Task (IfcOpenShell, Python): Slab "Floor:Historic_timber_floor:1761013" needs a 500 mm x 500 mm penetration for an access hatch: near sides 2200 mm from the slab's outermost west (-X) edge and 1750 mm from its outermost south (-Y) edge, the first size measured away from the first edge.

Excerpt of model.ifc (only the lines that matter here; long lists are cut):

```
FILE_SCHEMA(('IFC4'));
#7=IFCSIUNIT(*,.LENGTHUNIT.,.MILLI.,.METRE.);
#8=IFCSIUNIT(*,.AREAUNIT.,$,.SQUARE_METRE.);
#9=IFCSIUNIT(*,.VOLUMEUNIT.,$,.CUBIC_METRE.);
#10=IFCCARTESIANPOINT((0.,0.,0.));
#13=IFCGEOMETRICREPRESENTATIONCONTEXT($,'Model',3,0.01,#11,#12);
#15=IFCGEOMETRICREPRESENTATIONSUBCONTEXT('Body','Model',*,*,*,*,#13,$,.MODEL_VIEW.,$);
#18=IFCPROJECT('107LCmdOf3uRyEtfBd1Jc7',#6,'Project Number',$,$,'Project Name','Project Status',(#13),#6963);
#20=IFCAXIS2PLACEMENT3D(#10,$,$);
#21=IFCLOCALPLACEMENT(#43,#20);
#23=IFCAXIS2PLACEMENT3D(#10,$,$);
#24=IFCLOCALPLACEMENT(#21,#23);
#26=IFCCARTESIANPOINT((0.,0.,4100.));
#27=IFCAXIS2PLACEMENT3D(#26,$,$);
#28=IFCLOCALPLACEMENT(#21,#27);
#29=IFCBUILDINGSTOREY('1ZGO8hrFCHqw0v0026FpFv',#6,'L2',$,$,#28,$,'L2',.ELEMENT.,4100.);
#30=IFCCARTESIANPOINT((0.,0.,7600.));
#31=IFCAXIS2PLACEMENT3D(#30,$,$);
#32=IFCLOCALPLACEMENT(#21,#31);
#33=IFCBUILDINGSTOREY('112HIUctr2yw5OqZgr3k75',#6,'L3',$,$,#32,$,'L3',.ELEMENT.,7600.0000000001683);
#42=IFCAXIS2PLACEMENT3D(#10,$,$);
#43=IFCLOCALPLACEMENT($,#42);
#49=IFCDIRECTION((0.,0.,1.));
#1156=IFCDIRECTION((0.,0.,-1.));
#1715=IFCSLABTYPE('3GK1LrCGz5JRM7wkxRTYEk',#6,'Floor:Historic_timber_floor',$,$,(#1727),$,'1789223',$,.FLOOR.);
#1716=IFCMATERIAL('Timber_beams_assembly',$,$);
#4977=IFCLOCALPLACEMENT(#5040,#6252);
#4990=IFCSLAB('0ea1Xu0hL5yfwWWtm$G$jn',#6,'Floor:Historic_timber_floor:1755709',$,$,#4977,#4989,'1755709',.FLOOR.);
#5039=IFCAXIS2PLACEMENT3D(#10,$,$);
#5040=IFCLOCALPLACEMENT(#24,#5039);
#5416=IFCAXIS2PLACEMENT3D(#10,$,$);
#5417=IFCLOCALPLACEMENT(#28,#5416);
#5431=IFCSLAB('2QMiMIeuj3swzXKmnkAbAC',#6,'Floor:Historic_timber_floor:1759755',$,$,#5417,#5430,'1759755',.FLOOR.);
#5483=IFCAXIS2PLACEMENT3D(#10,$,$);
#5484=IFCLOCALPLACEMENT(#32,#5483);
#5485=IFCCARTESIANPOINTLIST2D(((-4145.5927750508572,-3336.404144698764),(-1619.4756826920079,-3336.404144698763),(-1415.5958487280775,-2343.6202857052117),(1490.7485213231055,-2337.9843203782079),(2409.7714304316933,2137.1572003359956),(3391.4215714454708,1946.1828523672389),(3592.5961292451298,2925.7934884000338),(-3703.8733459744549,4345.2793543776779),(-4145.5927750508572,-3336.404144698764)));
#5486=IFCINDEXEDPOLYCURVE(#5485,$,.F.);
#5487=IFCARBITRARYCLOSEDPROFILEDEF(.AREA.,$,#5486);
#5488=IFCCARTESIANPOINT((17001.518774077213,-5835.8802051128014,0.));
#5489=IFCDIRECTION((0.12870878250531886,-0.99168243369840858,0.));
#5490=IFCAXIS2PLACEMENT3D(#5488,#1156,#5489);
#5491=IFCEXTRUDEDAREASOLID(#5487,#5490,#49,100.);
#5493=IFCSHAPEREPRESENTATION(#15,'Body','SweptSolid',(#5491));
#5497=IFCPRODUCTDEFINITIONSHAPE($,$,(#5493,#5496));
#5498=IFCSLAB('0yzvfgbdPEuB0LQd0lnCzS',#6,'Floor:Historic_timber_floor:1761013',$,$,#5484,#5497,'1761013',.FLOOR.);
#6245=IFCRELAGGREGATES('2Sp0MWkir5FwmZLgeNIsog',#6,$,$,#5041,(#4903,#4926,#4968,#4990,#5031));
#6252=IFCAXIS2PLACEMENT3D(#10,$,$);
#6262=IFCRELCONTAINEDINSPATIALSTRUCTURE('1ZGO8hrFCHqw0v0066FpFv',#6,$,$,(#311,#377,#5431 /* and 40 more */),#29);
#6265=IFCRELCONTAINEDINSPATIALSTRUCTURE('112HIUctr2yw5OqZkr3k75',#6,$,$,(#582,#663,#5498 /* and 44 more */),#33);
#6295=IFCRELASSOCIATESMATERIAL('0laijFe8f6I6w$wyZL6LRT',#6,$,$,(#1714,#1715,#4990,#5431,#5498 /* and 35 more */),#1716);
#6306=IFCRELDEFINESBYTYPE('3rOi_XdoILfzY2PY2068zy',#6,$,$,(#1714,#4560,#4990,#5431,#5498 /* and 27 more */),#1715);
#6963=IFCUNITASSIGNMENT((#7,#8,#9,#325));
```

```python
import numpy as np
import ifcopenshell
import ifcopenshell.api.feature
import ifcopenshell.api.geometry
import ifcopenshell.api.root
import ifcopenshell.geom
import ifcopenshell.util.placement
import ifcopenshell.util.representation
import ifcopenshell.util.shape
import ifcopenshell.util.unit

model = ifcopenshell.open("model.ifc")
unit_scale = ifcopenshell.util.unit.calculate_unit_scale(model)
settings = ifcopenshell.geom.settings()


def volume(element):
    """Net volume in cubic metres, openings subtracted."""
    shape = ifcopenshell.geom.create_shape(settings, element)
    return ifcopenshell.util.shape.get_volume(shape.geometry)


slab = model.by_guid("0yzvfgbdPEuB0LQd0lnCzS")
before = volume(slab)

# Extent in the slab's own axes, in metres. The edges named are its -X and -Y sides.
slab_shape = ifcopenshell.geom.create_shape(settings, slab)
vertices = ifcopenshell.util.shape.get_vertices(slab_shape.geometry)
x_min, y_min, bottom = vertices.min(axis=0)
top = vertices[:, 2].max()

opening = ifcopenshell.api.root.create_entity(model, ifc_class="IfcOpeningElement", name="Access hatch opening", predefined_type="OPENING")
context = ifcopenshell.util.representation.get_context(model, "Model", "Body", "MODEL_VIEW")
width, depth = 0.5, 0.5
outline = [(0.0, 0.0), (width, 0.0), (width, depth), (0.0, depth), (0.0, 0.0)]
# Overshoot both faces by 50 mm so the cut is clean.
shape = ifcopenshell.api.geometry.add_slab_representation(
    model, context=context, depth=top - bottom + 0.1, polyline=outline
)
ifcopenshell.api.geometry.assign_representation(model, product=opening, representation=shape)

matrix = ifcopenshell.util.placement.get_local_placement(slab.ObjectPlacement)
matrix[:, 3] = matrix @ np.append(np.array([x_min + 2.2, y_min + 1.75, bottom - 0.05]) / unit_scale, 1.0)
ifcopenshell.api.geometry.edit_object_placement(model, product=opening, matrix=matrix, is_si=False)
ifcopenshell.api.feature.add_feature(model, feature=opening, element=slab)

after = volume(slab)

print(f"slab volume {before:.3f} -> {after:.3f} m3")

model.write("model-out.ifc")
```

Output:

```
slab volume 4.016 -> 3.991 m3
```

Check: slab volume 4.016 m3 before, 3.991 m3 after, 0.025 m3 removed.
